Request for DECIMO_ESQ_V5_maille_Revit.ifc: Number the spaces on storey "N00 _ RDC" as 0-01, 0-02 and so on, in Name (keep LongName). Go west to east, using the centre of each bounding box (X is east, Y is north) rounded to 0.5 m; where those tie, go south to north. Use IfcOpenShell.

First a look at what the model holds.

```python
import ifcopenshell
import ifcopenshell.util.element
import ifcopenshell.util.placement

model = ifcopenshell.open("DECIMO_ESQ_V5_maille_Revit.ifc")
print(model.schema)
storey = next(s for s in model.by_type("IfcBuildingStorey") if s.Name == "N00 _ RDC")
spaces = [e for e in ifcopenshell.util.element.get_decomposition(storey) if e.is_a("IfcSpace")]
for e in sorted(spaces, key=lambda e: e.id()):
    origin = ifcopenshell.util.placement.get_local_placement(e.ObjectPlacement)[:3, 3]
    print(e.id(), e.Name, e.LongName, origin.round(2) + 0.0, sep=" | ")
```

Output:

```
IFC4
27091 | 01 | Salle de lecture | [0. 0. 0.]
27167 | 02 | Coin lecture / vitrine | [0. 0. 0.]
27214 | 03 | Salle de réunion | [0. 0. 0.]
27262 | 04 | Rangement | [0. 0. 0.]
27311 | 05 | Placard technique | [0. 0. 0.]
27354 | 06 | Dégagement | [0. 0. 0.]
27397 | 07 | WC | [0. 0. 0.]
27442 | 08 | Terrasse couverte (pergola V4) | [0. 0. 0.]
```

```python
import ifcopenshell
import ifcopenshell.geom
import ifcopenshell.util.element
import ifcopenshell.util.shape

model = ifcopenshell.open("DECIMO_ESQ_V5_maille_Revit.ifc")
settings = ifcopenshell.geom.settings()
settings.set("use-world-coords", True)


def centre(element):
    shape = ifcopenshell.geom.create_shape(settings, element)
    return ifcopenshell.util.shape.get_bbox_centroid(shape.geometry)


storey = next(s for s in model.by_type("IfcBuildingStorey") if s.Name == "N00 _ RDC")
spaces = [e for e in ifcopenshell.util.element.get_decomposition(storey) if e.is_a("IfcSpace")]

# Insertion points can sit at a corner or the storey origin, so sort by the geometry (in metres).
centres = {e: centre(e) for e in spaces}
spaces.sort(key=lambda e: (round(centres[e][0] / 0.5), centres[e][1]))

for i, e in enumerate(spaces, start=1):
    number = f"0-{i:02d}"
    e.Name = number
    print(e.id(), number)

model.write("DECIMO_ESQ_V5_maille_Revit-out.ifc")
```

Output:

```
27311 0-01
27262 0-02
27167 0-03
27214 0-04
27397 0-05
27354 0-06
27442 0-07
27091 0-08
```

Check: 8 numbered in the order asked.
